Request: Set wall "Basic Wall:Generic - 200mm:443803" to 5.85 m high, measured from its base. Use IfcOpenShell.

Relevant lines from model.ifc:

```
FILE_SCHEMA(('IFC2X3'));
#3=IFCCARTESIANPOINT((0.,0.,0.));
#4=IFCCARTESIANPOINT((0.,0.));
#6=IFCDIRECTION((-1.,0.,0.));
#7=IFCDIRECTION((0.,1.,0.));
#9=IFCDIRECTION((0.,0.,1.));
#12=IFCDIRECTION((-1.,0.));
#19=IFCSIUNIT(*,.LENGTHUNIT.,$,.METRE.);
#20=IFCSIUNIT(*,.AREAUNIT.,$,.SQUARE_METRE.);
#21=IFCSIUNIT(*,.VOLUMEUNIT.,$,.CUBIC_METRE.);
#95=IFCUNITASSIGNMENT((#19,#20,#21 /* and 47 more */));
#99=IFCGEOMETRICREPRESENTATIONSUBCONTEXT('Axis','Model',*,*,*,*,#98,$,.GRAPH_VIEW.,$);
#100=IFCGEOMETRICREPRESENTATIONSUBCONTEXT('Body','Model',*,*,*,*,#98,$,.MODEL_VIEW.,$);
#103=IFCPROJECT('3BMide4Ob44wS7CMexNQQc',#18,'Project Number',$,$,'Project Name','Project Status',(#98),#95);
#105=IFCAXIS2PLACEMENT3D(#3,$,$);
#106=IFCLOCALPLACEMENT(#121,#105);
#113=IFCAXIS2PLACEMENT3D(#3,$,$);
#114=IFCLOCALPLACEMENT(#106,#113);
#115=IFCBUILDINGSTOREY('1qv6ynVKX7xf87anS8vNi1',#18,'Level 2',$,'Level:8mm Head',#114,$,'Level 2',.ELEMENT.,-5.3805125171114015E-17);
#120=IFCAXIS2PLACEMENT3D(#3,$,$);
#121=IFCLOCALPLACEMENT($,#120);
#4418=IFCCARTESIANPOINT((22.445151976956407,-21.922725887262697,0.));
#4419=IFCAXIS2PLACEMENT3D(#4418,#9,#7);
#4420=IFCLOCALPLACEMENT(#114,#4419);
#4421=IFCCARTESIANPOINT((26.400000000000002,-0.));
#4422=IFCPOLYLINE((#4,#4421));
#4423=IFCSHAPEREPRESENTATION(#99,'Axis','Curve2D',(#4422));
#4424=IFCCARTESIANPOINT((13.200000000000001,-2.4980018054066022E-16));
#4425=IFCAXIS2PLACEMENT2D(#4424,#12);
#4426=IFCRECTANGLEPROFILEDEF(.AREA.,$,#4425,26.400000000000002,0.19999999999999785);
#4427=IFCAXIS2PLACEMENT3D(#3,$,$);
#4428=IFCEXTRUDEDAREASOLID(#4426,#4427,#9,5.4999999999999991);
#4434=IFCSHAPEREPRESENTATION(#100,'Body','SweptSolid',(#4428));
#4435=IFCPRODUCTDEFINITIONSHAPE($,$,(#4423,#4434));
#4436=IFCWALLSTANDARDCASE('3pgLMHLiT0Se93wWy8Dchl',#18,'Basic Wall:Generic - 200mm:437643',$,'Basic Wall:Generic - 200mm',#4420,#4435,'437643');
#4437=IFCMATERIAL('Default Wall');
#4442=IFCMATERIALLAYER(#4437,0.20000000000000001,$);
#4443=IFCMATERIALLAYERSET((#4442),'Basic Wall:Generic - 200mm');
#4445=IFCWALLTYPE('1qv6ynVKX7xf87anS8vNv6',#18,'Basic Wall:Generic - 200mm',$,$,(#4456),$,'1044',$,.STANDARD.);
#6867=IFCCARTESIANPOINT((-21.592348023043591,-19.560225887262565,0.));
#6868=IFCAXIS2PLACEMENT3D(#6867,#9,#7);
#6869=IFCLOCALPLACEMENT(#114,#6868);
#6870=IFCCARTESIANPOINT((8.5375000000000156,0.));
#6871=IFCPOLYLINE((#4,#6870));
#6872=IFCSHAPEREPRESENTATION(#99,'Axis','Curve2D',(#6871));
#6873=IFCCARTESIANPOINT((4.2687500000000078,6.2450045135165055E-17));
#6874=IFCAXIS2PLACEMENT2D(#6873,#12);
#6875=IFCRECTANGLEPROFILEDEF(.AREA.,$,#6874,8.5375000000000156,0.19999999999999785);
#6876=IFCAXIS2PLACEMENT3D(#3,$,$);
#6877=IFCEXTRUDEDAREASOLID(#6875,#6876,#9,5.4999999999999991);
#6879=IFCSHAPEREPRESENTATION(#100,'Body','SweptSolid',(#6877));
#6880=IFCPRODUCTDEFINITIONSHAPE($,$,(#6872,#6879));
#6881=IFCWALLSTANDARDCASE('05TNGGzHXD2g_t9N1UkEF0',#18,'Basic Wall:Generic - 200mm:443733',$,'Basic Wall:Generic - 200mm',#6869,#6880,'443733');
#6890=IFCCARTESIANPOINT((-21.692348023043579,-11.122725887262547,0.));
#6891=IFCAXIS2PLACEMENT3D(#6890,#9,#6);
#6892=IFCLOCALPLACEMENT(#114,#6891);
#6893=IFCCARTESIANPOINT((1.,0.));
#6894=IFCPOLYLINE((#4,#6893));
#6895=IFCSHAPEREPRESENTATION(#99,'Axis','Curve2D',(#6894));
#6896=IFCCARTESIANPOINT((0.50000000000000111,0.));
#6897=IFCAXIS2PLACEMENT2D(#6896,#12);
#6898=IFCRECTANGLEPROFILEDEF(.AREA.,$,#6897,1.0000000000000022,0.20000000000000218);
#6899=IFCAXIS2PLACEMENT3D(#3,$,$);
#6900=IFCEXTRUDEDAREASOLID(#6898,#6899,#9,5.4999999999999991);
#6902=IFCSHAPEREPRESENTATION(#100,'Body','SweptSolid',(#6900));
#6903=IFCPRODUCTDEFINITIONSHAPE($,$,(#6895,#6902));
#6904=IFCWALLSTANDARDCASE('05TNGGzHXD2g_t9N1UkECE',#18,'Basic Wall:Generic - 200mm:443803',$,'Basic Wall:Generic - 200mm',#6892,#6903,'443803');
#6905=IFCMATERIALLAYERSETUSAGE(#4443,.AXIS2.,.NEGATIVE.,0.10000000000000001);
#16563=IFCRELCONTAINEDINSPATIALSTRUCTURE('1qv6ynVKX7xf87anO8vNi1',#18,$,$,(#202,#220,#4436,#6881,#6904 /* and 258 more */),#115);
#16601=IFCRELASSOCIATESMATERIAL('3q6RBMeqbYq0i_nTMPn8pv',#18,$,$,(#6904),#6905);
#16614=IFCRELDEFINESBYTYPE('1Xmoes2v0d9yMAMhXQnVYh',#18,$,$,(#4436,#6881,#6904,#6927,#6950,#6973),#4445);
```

```python
import ifcopenshell
import ifcopenshell.geom
import ifcopenshell.util.representation
import ifcopenshell.util.shape

model = ifcopenshell.open("model.ifc")
settings = ifcopenshell.geom.settings()


def volume(element):
    """Net volume in cubic metres, openings subtracted."""
    shape = ifcopenshell.geom.create_shape(settings, element)
    return ifcopenshell.util.shape.get_volume(shape.geometry)


wall = model.by_guid("05TNGGzHXD2g_t9N1UkECE")
before = volume(wall)

body = ifcopenshell.util.representation.get_representation(wall, "Model", "Body")
solid = body.Items[0]
old_height = solid.Depth
solid.Depth = 5.85
after = volume(wall)

print(f"height {old_height:g} -> {solid.Depth:g}, volume {before:.3f} -> {after:.3f} m3")

model.write("model_edited.ifc")
```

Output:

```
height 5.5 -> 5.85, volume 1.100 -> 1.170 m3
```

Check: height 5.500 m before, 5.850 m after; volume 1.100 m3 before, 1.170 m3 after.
